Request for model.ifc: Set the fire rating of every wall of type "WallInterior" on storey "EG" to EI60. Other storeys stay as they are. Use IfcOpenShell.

First a look at what the model holds.

```python
import ifcopenshell
import ifcopenshell.util.element

model = ifcopenshell.open("model.ifc")
print(model.schema)
storey = next(s for s in model.by_type("IfcBuildingStorey") if s.Name == "EG")
walls = [e for e in ifcopenshell.util.element.get_decomposition(storey) if e.is_a("IfcWall")]
seen = {}
for e in walls:
    element_type = ifcopenshell.util.element.get_type(e)
    key = (element_type.Name if element_type != e and element_type else None, ifcopenshell.util.element.get_pset(e, "Pset_WallCommon", "FireRating"))
    seen[key] = seen.get(key, 0) + 1
for (name, value), count in sorted(seen.items(), key=str):
    print(count, "x", name, "|", value)
```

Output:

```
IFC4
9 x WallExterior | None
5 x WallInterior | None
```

```python
import ifcopenshell
import ifcopenshell.api.pset
import ifcopenshell.util.element

model = ifcopenshell.open("model.ifc")

storey = next(s for s in model.by_type("IfcBuildingStorey") if s.Name == "EG")
walls = [e for e in ifcopenshell.util.element.get_decomposition(storey) if e.is_a("IfcWall")]

count = 0
for e in walls:
    element_type = ifcopenshell.util.element.get_type(e)
    if element_type in (None, e) or element_type.Name != "WallInterior":
        continue
    # add_pset returns the element's existing set when there is one.
    pset = ifcopenshell.api.pset.add_pset(model, product=e, name="Pset_WallCommon")
    ifcopenshell.api.pset.edit_pset(model, pset=pset, properties={"FireRating": "EI60"})
    count += 1

print(count, "walls updated")

model.write("model_edited.ifc")
```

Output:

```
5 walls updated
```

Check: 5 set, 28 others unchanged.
